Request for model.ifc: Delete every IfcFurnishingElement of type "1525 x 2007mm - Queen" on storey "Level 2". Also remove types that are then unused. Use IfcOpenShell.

First a look at what the model holds.

```python
import ifcopenshell
import ifcopenshell.util.element

model = ifcopenshell.open("model.ifc")
print(model.schema)
storey = next(s for s in model.by_type("IfcBuildingStorey") if s.Name == "Level 2")
furniture = [e for e in ifcopenshell.util.element.get_decomposition(storey) if e.is_a("IfcFurnishingElement")]
seen = {}
for e in furniture:
    element_type = ifcopenshell.util.element.get_type(e)
    name = element_type.Name if element_type not in (None, e) else None
    seen[name] = seen.get(name, 0) + 1
for name, count in sorted(seen.items(), key=str):
    print(count, "x", name)
```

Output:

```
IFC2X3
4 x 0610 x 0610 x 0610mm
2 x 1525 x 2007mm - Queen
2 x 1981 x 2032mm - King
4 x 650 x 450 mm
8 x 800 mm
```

```python
import ifcopenshell
import ifcopenshell.api.root
import ifcopenshell.util.element

model = ifcopenshell.open("model.ifc")

storey = next(s for s in model.by_type("IfcBuildingStorey") if s.Name == "Level 2")
furniture = [e for e in ifcopenshell.util.element.get_decomposition(storey) if e.is_a("IfcFurnishingElement")]
targets = [e for e in furniture if (t := ifcopenshell.util.element.get_type(e)) not in (None, e) and t.Name == "1525 x 2007mm - Queen"]
types = {ifcopenshell.util.element.get_type(e) for e in targets} - {None, *targets}

for e in targets:
    ifcopenshell.api.root.remove_product(model, product=e)
print(len(targets), "removed")

unused = [t for t in types if not ifcopenshell.util.element.get_types(t)]
for t in unused:
    ifcopenshell.api.root.remove_product(model, product=t)
print(len(unused), "unused types removed")

model.write("model_v2.ifc")
```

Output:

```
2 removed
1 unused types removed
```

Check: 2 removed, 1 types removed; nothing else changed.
